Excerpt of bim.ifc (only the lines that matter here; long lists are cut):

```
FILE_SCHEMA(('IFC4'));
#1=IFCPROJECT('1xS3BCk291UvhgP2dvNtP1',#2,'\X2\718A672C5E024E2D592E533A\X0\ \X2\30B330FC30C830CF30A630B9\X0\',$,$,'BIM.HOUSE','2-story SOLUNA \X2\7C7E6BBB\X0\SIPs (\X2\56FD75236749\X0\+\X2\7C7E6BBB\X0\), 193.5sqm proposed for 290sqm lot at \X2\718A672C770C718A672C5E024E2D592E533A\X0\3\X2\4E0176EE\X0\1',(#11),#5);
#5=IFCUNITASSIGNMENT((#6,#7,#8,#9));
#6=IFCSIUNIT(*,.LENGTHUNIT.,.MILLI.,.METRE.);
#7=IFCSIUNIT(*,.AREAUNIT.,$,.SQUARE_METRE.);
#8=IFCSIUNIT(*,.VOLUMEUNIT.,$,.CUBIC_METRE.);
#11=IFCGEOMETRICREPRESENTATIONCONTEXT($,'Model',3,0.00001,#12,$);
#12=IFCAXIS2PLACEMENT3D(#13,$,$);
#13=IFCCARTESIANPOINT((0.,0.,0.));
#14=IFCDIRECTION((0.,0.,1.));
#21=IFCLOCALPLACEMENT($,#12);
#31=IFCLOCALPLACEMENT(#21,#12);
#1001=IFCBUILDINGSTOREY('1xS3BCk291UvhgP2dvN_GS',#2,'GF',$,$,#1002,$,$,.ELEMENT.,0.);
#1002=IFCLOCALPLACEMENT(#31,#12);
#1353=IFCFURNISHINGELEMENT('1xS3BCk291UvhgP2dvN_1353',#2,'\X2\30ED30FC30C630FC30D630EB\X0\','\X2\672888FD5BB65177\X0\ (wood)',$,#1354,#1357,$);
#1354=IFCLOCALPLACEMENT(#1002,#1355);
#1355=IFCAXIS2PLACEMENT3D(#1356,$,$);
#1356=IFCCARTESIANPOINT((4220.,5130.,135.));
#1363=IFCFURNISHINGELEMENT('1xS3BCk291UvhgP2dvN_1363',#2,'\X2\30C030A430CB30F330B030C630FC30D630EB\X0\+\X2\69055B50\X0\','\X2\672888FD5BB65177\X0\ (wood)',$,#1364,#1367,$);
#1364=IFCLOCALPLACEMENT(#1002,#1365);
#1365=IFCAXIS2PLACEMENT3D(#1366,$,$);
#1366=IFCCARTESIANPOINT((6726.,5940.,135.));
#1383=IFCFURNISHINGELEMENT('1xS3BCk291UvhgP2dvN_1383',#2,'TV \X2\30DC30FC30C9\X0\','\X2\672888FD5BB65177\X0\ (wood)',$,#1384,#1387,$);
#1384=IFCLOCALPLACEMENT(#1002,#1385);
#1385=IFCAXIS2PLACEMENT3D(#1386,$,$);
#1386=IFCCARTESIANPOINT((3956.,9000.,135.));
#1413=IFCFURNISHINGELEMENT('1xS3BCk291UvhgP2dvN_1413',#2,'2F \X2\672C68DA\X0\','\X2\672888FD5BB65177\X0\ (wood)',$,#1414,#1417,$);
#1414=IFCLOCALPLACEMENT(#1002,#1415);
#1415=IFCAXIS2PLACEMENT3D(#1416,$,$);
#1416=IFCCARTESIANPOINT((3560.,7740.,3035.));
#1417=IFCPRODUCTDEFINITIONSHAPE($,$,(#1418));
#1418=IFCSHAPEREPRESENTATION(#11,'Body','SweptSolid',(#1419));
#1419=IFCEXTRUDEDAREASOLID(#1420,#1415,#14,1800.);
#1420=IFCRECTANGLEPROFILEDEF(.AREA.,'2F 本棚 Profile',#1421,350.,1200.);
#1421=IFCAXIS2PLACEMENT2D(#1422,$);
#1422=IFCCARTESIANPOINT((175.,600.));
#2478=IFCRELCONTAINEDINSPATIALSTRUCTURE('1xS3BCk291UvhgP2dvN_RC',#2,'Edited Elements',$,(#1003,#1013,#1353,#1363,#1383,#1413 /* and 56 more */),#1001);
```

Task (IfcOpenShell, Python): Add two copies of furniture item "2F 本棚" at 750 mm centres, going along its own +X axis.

```python
import ifcopenshell
import ifcopenshell.api.geometry
import ifcopenshell.api.root
import ifcopenshell.util.element
import ifcopenshell.util.placement
import ifcopenshell.util.unit

model = ifcopenshell.open("bim.ifc")
unit_scale = ifcopenshell.util.unit.calculate_unit_scale(model)


def reuse_history(source, copy):
    """copy_class also copies each property set's owner history, people and application; keep the originals."""
    for rel in copy.IsDefinedBy:
        if rel.is_a("IfcRelDefinesByProperties") and (history := rel.RelatingPropertyDefinition.OwnerHistory):
            rel.RelatingPropertyDefinition.OwnerHistory = source.OwnerHistory
            ifcopenshell.util.element.remove_deep2(model, history)


source = model.by_guid("1xS3BCk291UvhgP2dvN_1413")
base = ifcopenshell.util.placement.get_local_placement(source.ObjectPlacement)
step = base[:3, 0] * 0.75 / unit_scale

for i in range(1, 3):
    copy = ifcopenshell.api.root.copy_class(model, product=source)
    copy.Representation = ifcopenshell.util.element.copy_deep(
        model, source.Representation, exclude=["IfcGeometricRepresentationContext", "IfcRepresentationMap"]
    )
    reuse_history(source, copy)
    matrix = base.copy()
    matrix[:3, 3] += i * step
    print("added at", matrix[:3, 3].round(3) + 0.0)
    ifcopenshell.api.geometry.edit_object_placement(model, product=copy, matrix=matrix, is_si=False)

model.write("bim_edited.ifc")
```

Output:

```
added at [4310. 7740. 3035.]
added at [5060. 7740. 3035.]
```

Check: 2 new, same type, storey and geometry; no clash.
